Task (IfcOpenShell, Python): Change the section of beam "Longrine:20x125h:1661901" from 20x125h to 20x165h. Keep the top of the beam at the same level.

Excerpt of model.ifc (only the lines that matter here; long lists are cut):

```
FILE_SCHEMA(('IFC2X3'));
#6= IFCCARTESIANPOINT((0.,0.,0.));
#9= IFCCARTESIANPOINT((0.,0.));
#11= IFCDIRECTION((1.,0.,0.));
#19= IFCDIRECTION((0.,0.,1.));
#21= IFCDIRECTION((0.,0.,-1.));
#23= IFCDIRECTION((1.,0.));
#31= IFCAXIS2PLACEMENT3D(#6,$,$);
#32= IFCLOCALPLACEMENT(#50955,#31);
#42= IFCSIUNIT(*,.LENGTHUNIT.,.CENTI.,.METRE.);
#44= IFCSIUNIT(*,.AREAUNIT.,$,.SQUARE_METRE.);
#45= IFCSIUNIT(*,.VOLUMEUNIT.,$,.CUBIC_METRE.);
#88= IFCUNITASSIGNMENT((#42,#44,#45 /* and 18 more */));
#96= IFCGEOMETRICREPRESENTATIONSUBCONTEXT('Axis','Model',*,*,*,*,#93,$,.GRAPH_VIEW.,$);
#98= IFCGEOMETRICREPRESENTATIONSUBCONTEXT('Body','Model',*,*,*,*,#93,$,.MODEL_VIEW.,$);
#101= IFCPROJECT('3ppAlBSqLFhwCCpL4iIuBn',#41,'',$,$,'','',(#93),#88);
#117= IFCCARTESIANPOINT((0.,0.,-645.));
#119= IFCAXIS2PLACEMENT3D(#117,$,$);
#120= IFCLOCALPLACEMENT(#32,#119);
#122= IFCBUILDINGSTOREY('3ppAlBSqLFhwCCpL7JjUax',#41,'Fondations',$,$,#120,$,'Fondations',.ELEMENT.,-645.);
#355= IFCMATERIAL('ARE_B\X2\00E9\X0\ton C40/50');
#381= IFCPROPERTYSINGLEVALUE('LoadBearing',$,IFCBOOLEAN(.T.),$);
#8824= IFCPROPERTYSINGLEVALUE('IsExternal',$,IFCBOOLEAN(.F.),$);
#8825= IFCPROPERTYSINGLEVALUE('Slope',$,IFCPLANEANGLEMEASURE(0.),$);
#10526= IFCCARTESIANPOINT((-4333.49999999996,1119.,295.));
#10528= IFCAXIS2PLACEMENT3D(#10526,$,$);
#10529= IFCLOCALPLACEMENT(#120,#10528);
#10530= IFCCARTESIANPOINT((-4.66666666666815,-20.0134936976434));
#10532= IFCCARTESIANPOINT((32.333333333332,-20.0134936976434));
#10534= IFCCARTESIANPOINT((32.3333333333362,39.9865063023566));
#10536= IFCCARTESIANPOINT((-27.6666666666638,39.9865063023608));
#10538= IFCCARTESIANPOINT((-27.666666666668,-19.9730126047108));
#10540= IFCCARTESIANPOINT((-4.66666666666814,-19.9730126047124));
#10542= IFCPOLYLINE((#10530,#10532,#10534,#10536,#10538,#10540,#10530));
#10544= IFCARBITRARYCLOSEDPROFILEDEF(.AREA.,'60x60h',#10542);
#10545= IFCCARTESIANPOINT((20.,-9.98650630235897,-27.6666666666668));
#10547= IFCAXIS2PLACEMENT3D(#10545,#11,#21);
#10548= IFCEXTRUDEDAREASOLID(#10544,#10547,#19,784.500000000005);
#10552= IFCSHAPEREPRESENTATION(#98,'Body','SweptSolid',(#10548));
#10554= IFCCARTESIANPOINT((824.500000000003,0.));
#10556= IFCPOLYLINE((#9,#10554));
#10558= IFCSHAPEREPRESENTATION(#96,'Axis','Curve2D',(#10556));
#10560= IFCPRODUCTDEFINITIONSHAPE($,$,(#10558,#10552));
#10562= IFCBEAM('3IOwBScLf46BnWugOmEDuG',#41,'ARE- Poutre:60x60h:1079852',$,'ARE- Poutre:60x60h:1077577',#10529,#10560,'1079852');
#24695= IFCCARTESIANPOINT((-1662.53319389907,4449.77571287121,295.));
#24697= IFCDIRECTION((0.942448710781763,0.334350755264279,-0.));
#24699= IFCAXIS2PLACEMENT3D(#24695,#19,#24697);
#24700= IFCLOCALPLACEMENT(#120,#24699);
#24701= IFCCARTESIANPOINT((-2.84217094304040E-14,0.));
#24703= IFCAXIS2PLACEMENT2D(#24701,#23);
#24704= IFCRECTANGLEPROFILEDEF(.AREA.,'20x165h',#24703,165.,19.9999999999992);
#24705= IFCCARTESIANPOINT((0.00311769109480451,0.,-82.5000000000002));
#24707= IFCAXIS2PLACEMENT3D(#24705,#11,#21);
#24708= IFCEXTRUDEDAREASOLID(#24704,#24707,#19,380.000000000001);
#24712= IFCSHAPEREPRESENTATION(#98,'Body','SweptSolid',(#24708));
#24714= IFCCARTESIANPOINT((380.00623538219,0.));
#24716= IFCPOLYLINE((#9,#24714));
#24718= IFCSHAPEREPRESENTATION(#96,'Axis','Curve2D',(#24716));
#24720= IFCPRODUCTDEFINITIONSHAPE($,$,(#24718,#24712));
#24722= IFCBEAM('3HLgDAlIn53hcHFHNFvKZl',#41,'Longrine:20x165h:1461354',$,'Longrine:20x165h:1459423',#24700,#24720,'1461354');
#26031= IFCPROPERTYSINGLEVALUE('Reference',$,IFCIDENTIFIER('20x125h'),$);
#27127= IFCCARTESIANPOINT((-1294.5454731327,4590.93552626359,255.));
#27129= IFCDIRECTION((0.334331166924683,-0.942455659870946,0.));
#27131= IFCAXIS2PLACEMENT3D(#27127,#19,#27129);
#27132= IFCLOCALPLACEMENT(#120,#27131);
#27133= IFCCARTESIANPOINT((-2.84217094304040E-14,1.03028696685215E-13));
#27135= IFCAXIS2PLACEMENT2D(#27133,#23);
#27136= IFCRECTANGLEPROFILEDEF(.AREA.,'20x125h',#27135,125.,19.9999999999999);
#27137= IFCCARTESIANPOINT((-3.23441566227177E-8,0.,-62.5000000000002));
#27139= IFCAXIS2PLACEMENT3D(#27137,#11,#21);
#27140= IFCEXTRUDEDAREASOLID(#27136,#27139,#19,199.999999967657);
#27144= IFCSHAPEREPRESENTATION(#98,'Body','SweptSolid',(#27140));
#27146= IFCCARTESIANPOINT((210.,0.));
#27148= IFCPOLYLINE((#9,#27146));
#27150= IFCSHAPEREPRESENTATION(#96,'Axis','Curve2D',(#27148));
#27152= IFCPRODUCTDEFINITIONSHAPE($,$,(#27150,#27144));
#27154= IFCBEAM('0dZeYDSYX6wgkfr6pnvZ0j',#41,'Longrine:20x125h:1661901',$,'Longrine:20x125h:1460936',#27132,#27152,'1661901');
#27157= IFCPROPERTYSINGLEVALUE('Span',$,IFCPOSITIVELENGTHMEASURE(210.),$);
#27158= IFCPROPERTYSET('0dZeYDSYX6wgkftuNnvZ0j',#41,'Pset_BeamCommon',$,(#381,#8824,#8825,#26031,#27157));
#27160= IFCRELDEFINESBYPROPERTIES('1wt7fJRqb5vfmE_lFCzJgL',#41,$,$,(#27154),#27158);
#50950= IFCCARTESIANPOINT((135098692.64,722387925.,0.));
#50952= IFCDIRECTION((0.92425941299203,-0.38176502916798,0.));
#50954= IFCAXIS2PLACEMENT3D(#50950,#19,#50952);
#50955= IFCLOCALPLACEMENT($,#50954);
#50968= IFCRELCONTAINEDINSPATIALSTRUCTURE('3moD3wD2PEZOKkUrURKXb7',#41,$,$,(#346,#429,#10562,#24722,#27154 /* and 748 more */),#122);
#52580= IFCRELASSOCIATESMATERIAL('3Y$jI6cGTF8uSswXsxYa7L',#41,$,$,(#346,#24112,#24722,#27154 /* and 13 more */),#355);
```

```python
import ifcopenshell
import ifcopenshell.api.pset
import ifcopenshell.util.element
import ifcopenshell.util.representation

model = ifcopenshell.open("model.ifc")

member = model.by_guid("0dZeYDSYX6wgkfr6pnvZ0j")
source = next(p for p in model.by_type("IfcRectangleProfileDef") if p.ProfileName == "20x165h")

body = ifcopenshell.util.representation.get_representation(member, "Model", "Body")
solid = body.Items[0]
old_profile = solid.SweptArea

# Copy the section's sizes but keep this member's own profile position.
profile = ifcopenshell.util.element.copy(model, source)
# Profiles are centred, so shift by half the change in depth to hold the top.
shift = (old_profile.XDim - profile.XDim) / 2
x, y = old_profile.Position.Location.Coordinates
up = (-1.0, 0.0)  # upwards, in the solid's own plane
location = model.createIfcCartesianPoint((x + up[0] * shift, y + up[1] * shift))
profile.Position = model.createIfcAxis2Placement2D(location, old_profile.Position.RefDirection)
solid.SweptArea = profile
if not model.get_total_inverses(old_profile):
    ifcopenshell.util.element.remove_deep2(model, old_profile)
member.Name = member.Name.replace("20x125h", "20x165h")
member.ObjectType = member.ObjectType.replace("20x125h", "20x165h")
pset = model.by_id(ifcopenshell.util.element.get_pset(member, "Pset_BeamCommon", should_inherit=False)["id"])
ifcopenshell.api.pset.edit_pset(model, pset=pset, properties={"Reference": "20x165h"})

print(solid.SweptArea)

model.write("model_rev.ifc")
```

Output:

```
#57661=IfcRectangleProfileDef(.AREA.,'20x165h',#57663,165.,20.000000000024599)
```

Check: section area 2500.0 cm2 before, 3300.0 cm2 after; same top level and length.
